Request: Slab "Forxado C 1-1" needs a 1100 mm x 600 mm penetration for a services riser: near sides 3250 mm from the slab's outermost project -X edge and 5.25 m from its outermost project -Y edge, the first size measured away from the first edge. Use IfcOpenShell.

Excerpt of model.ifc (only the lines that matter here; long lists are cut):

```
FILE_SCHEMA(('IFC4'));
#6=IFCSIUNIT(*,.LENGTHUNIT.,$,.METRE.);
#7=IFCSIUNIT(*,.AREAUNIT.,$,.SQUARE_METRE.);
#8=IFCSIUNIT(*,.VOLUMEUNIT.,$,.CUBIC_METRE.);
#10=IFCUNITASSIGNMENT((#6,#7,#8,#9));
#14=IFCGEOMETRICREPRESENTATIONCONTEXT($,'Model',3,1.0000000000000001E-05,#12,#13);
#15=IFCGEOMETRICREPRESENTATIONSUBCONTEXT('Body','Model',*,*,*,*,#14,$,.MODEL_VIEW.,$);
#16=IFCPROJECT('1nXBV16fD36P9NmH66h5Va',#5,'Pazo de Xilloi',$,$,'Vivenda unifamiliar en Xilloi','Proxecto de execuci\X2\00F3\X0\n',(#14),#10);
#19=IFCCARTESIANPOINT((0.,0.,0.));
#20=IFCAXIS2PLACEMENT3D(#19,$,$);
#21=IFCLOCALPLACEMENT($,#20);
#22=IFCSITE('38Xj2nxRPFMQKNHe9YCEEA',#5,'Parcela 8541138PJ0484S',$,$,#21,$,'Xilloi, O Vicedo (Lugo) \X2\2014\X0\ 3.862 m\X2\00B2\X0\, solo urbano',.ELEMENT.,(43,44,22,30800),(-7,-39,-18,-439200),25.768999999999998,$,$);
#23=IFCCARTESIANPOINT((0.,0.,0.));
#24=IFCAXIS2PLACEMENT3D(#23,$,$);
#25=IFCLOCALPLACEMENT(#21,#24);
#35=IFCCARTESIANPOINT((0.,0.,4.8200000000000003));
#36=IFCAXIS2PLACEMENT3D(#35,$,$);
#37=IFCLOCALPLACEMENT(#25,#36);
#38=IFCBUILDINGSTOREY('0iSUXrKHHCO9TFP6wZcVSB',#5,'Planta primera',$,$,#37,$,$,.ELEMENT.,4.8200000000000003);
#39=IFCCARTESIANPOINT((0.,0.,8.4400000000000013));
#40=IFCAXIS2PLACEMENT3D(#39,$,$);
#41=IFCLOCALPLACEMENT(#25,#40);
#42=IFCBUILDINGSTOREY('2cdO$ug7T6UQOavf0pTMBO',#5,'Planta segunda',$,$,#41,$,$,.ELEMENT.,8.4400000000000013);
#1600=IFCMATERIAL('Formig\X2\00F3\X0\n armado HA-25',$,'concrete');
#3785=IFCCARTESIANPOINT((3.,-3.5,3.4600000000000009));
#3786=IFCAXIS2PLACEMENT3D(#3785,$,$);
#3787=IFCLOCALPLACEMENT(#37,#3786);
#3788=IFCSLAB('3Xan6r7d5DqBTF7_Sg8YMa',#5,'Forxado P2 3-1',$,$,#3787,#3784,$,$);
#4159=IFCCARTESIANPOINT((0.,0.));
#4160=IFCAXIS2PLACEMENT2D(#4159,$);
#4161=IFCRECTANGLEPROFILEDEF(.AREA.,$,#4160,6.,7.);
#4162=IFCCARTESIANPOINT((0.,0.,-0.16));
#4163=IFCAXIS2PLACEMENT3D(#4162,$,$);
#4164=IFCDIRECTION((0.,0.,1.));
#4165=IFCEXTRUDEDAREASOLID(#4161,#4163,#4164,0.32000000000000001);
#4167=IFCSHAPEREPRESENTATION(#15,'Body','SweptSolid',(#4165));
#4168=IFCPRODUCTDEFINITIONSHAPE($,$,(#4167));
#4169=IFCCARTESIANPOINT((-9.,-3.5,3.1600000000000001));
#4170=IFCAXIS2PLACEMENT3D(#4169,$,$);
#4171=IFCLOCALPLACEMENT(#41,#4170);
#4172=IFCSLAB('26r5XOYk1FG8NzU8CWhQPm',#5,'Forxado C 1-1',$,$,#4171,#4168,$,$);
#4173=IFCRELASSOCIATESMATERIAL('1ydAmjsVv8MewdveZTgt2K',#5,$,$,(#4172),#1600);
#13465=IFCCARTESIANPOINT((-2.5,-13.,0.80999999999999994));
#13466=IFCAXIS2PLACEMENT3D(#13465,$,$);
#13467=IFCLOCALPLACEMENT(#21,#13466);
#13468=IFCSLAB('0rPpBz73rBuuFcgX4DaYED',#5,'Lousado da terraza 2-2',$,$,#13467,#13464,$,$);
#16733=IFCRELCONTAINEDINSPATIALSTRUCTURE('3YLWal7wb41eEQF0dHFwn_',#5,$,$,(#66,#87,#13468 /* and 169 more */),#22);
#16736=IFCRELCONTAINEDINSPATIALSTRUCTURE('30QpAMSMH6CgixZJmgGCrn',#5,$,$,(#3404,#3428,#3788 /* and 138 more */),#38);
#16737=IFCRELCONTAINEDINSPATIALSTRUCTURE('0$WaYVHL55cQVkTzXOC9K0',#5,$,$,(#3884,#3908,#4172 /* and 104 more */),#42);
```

```python
import numpy as np
import ifcopenshell
import ifcopenshell.api.feature
import ifcopenshell.api.geometry
import ifcopenshell.api.root
import ifcopenshell.geom
import ifcopenshell.util.placement
import ifcopenshell.util.representation
import ifcopenshell.util.shape
import ifcopenshell.util.unit

model = ifcopenshell.open("model.ifc")
unit_scale = ifcopenshell.util.unit.calculate_unit_scale(model)
settings = ifcopenshell.geom.settings()


def volume(element):
    """Net volume in cubic metres, openings subtracted."""
    shape = ifcopenshell.geom.create_shape(settings, element)
    return ifcopenshell.util.shape.get_volume(shape.geometry)


slab = model.by_guid("26r5XOYk1FG8NzU8CWhQPm")
before = volume(slab)

# Extent in the slab's own axes, in metres. The edges named are its -X and -Y sides.
slab_shape = ifcopenshell.geom.create_shape(settings, slab)
vertices = ifcopenshell.util.shape.get_vertices(slab_shape.geometry)
x_min, y_min, bottom = vertices.min(axis=0)
top = vertices[:, 2].max()

opening = ifcopenshell.api.root.create_entity(model, ifc_class="IfcOpeningElement", name="Services riser opening", predefined_type="OPENING")
context = ifcopenshell.util.representation.get_context(model, "Model", "Body", "MODEL_VIEW")
width, depth = 1.1, 0.6
outline = [(0.0, 0.0), (width, 0.0), (width, depth), (0.0, depth), (0.0, 0.0)]
# Overshoot both faces by 50 mm so the cut is clean.
shape = ifcopenshell.api.geometry.add_slab_representation(
    model, context=context, depth=top - bottom + 0.1, polyline=outline
)
ifcopenshell.api.geometry.assign_representation(model, product=opening, representation=shape)

matrix = ifcopenshell.util.placement.get_local_placement(slab.ObjectPlacement)
matrix[:, 3] = matrix @ np.append(np.array([x_min + 3.25, y_min + 5.25, bottom - 0.05]) / unit_scale, 1.0)
ifcopenshell.api.geometry.edit_object_placement(model, product=opening, matrix=matrix, is_si=False)
ifcopenshell.api.feature.add_feature(model, feature=opening, element=slab)

after = volume(slab)

print(f"slab volume {before:.3f} -> {after:.3f} m3")

model.write("model_rev.ifc")
```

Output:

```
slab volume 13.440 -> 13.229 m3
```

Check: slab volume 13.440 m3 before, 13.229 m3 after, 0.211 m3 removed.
